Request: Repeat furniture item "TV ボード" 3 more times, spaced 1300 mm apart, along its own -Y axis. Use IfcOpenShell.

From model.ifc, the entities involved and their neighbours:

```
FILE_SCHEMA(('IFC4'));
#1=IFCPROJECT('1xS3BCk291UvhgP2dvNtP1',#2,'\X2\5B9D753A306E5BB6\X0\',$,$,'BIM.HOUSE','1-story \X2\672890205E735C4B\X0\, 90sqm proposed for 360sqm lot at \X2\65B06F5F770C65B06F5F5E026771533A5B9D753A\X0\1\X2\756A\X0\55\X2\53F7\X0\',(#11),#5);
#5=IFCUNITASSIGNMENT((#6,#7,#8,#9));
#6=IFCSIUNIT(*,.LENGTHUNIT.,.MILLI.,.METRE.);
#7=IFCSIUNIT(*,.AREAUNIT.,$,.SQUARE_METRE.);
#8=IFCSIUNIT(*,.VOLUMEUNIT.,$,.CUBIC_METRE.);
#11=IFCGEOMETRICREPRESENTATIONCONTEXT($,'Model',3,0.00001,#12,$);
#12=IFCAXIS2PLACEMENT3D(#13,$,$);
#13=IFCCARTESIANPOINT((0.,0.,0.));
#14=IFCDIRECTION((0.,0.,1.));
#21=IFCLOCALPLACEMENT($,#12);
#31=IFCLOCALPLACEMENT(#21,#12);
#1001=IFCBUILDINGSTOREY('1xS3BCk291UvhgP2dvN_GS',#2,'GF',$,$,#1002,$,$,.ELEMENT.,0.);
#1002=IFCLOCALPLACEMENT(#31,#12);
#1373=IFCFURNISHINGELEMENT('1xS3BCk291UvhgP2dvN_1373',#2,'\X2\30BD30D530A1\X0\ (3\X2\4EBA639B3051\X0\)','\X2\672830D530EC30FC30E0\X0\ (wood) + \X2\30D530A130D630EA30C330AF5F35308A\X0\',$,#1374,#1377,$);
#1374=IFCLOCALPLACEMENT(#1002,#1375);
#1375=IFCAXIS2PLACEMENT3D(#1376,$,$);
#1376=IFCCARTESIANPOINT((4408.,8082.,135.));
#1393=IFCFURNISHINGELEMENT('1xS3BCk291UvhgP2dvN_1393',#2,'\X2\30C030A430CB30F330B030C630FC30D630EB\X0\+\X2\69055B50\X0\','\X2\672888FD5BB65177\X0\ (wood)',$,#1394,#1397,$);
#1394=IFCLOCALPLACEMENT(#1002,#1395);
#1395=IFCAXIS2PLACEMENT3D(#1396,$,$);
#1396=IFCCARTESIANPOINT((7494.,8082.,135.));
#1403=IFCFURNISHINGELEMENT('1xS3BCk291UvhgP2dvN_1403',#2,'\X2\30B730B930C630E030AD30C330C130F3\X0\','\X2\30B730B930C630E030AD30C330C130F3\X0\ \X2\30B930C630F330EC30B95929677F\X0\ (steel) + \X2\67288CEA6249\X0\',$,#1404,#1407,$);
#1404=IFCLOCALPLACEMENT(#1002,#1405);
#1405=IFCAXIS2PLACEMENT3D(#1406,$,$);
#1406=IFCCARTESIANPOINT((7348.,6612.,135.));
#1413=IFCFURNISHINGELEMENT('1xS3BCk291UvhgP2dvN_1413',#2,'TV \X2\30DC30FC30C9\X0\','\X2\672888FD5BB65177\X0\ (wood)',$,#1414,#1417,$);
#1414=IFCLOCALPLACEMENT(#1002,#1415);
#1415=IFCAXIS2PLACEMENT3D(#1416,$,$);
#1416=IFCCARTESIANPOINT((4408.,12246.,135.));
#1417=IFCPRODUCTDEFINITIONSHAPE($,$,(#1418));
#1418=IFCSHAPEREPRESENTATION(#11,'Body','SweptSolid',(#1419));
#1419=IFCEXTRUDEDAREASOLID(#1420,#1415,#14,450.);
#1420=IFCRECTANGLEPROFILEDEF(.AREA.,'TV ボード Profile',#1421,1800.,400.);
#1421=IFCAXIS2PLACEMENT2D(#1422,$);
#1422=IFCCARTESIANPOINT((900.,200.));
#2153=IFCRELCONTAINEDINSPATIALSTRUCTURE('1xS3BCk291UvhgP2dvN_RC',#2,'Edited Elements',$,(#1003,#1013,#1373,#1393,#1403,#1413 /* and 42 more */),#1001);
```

```python
import ifcopenshell
import ifcopenshell.api.geometry
import ifcopenshell.api.root
import ifcopenshell.util.element
import ifcopenshell.util.placement
import ifcopenshell.util.unit

model = ifcopenshell.open("model.ifc")
unit_scale = ifcopenshell.util.unit.calculate_unit_scale(model)


def reuse_history(source, copy):
    """copy_class also copies each property set's owner history, people and application; keep the originals."""
    for rel in copy.IsDefinedBy:
        if rel.is_a("IfcRelDefinesByProperties") and (history := rel.RelatingPropertyDefinition.OwnerHistory):
            rel.RelatingPropertyDefinition.OwnerHistory = source.OwnerHistory
            ifcopenshell.util.element.remove_deep2(model, history)


source = model.by_id(1413)
base = ifcopenshell.util.placement.get_local_placement(source.ObjectPlacement)
step = -base[:3, 1] * 1.3 / unit_scale

for i in range(1, 4):
    copy = ifcopenshell.api.root.copy_class(model, product=source)
    copy.Representation = ifcopenshell.util.element.copy_deep(
        model, source.Representation, exclude=["IfcGeometricRepresentationContext", "IfcRepresentationMap"]
    )
    reuse_history(source, copy)
    matrix = base.copy()
    matrix[:3, 3] += i * step
    print("added at", matrix[:3, 3].round(3) + 0.0)
    ifcopenshell.api.geometry.edit_object_placement(model, product=copy, matrix=matrix, is_si=False)

model.write("model_v2.ifc")
```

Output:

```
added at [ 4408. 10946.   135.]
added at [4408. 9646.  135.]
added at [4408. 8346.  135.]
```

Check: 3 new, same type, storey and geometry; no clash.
